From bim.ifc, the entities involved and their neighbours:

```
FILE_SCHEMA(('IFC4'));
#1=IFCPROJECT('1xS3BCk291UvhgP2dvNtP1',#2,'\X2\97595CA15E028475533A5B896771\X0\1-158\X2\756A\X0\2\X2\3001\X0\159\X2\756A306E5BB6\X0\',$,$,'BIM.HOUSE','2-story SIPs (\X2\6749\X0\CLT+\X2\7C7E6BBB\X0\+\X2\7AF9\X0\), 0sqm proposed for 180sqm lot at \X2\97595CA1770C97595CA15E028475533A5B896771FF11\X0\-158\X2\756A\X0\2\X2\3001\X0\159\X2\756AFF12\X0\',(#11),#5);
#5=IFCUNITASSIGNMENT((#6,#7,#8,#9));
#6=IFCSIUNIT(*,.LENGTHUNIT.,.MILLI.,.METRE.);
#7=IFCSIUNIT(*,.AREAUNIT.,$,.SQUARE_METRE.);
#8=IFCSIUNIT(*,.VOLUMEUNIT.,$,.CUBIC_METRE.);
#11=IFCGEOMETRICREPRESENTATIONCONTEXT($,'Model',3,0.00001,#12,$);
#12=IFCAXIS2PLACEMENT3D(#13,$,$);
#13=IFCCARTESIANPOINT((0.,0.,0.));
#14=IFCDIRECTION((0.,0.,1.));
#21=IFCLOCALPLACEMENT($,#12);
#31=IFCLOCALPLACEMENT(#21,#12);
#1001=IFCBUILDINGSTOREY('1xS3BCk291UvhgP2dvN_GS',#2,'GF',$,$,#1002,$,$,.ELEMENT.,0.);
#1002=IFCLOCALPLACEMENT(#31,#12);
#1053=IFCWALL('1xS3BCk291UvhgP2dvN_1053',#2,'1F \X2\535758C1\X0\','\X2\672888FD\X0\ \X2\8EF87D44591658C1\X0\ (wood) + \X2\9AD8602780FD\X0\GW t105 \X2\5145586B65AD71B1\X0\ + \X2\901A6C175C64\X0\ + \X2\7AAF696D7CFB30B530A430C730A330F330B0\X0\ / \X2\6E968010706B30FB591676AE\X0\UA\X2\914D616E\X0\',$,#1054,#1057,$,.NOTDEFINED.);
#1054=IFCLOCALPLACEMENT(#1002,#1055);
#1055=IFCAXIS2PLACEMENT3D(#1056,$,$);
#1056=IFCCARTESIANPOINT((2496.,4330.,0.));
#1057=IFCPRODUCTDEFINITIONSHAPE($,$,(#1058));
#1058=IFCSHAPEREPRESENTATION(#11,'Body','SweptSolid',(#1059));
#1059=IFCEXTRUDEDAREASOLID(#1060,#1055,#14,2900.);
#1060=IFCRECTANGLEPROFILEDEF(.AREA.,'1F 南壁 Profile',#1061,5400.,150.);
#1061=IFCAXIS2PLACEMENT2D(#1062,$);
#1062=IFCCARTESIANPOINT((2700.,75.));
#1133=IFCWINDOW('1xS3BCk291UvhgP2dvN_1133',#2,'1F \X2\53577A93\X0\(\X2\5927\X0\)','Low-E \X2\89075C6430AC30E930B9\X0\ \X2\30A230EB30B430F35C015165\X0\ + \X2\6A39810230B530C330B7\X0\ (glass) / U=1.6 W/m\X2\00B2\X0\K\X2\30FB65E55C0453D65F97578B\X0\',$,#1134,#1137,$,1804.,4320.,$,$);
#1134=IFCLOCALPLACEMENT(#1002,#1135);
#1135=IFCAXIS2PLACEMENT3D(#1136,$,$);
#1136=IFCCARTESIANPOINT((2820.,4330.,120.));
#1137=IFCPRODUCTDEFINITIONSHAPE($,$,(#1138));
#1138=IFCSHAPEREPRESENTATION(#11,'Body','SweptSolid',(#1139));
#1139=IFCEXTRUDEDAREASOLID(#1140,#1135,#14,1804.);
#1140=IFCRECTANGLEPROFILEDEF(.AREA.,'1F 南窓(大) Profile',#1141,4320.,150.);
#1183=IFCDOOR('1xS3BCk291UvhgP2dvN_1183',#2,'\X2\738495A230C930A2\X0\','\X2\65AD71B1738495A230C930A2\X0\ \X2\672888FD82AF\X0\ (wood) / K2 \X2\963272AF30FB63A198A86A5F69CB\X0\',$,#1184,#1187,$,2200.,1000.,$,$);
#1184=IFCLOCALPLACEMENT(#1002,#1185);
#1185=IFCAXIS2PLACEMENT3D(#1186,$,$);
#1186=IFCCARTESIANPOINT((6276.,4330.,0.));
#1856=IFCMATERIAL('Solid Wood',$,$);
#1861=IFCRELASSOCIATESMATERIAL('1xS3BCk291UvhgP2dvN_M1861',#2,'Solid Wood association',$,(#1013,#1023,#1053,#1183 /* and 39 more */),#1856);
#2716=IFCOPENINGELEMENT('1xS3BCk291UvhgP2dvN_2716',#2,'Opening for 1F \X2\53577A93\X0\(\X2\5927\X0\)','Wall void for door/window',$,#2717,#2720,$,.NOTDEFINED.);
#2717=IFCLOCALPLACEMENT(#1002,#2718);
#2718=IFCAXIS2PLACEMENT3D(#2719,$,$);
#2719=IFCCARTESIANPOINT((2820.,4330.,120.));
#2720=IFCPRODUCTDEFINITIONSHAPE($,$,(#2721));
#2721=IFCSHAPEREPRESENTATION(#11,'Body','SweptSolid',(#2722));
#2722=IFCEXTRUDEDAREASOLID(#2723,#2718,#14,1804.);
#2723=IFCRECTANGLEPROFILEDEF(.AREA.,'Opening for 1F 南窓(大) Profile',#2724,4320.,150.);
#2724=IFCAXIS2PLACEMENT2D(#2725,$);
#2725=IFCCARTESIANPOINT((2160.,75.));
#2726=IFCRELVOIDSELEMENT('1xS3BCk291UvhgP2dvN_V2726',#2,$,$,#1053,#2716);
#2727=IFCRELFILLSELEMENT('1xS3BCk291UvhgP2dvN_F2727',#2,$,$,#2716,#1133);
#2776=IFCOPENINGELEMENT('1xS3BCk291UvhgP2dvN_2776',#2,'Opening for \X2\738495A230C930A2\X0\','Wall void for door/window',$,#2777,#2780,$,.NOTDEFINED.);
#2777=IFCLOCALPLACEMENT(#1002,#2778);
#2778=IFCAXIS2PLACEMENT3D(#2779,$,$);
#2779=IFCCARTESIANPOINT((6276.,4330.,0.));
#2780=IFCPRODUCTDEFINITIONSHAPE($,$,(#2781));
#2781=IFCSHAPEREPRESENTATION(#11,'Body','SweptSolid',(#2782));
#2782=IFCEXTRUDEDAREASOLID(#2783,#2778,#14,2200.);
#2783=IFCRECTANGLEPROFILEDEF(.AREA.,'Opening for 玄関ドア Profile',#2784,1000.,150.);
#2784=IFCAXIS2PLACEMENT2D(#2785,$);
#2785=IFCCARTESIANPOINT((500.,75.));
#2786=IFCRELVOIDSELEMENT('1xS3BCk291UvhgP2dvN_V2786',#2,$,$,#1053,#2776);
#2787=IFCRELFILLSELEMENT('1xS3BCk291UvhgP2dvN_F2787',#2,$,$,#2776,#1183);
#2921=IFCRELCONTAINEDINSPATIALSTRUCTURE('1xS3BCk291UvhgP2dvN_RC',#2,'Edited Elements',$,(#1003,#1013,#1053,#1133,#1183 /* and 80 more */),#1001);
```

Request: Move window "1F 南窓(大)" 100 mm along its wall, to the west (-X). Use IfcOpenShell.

```python
import ifcopenshell
import ifcopenshell.api.geometry
import ifcopenshell.util.placement
import ifcopenshell.util.unit

model = ifcopenshell.open("bim.ifc")
unit_scale = ifcopenshell.util.unit.calculate_unit_scale(model)

window = model.by_guid("1xS3BCk291UvhgP2dvN_1133")
opening = window.FillsVoids[0].RelatingOpeningElement
wall = opening.VoidsElements[0].RelatingBuildingElement

wall_matrix = ifcopenshell.util.placement.get_local_placement(wall.ObjectPlacement)
shift = wall_matrix[:3, 0] * -0.1 / unit_scale
before = ifcopenshell.util.placement.get_local_placement(window.ObjectPlacement)[:3, 3].copy()

# The window is not placed relative to its opening, so move both.
for product in (opening, window):
    matrix = ifcopenshell.util.placement.get_local_placement(product.ObjectPlacement)
    matrix[:3, 3] += shift
    ifcopenshell.api.geometry.edit_object_placement(model, product=product, matrix=matrix, is_si=False)

after = ifcopenshell.util.placement.get_local_placement(window.ObjectPlacement)[:3, 3]
print("window moved by", (after - before).round(3) + 0.0)

model.write("bim_updated.ifc")
```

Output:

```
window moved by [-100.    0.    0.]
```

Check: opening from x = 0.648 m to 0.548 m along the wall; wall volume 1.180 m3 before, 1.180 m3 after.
